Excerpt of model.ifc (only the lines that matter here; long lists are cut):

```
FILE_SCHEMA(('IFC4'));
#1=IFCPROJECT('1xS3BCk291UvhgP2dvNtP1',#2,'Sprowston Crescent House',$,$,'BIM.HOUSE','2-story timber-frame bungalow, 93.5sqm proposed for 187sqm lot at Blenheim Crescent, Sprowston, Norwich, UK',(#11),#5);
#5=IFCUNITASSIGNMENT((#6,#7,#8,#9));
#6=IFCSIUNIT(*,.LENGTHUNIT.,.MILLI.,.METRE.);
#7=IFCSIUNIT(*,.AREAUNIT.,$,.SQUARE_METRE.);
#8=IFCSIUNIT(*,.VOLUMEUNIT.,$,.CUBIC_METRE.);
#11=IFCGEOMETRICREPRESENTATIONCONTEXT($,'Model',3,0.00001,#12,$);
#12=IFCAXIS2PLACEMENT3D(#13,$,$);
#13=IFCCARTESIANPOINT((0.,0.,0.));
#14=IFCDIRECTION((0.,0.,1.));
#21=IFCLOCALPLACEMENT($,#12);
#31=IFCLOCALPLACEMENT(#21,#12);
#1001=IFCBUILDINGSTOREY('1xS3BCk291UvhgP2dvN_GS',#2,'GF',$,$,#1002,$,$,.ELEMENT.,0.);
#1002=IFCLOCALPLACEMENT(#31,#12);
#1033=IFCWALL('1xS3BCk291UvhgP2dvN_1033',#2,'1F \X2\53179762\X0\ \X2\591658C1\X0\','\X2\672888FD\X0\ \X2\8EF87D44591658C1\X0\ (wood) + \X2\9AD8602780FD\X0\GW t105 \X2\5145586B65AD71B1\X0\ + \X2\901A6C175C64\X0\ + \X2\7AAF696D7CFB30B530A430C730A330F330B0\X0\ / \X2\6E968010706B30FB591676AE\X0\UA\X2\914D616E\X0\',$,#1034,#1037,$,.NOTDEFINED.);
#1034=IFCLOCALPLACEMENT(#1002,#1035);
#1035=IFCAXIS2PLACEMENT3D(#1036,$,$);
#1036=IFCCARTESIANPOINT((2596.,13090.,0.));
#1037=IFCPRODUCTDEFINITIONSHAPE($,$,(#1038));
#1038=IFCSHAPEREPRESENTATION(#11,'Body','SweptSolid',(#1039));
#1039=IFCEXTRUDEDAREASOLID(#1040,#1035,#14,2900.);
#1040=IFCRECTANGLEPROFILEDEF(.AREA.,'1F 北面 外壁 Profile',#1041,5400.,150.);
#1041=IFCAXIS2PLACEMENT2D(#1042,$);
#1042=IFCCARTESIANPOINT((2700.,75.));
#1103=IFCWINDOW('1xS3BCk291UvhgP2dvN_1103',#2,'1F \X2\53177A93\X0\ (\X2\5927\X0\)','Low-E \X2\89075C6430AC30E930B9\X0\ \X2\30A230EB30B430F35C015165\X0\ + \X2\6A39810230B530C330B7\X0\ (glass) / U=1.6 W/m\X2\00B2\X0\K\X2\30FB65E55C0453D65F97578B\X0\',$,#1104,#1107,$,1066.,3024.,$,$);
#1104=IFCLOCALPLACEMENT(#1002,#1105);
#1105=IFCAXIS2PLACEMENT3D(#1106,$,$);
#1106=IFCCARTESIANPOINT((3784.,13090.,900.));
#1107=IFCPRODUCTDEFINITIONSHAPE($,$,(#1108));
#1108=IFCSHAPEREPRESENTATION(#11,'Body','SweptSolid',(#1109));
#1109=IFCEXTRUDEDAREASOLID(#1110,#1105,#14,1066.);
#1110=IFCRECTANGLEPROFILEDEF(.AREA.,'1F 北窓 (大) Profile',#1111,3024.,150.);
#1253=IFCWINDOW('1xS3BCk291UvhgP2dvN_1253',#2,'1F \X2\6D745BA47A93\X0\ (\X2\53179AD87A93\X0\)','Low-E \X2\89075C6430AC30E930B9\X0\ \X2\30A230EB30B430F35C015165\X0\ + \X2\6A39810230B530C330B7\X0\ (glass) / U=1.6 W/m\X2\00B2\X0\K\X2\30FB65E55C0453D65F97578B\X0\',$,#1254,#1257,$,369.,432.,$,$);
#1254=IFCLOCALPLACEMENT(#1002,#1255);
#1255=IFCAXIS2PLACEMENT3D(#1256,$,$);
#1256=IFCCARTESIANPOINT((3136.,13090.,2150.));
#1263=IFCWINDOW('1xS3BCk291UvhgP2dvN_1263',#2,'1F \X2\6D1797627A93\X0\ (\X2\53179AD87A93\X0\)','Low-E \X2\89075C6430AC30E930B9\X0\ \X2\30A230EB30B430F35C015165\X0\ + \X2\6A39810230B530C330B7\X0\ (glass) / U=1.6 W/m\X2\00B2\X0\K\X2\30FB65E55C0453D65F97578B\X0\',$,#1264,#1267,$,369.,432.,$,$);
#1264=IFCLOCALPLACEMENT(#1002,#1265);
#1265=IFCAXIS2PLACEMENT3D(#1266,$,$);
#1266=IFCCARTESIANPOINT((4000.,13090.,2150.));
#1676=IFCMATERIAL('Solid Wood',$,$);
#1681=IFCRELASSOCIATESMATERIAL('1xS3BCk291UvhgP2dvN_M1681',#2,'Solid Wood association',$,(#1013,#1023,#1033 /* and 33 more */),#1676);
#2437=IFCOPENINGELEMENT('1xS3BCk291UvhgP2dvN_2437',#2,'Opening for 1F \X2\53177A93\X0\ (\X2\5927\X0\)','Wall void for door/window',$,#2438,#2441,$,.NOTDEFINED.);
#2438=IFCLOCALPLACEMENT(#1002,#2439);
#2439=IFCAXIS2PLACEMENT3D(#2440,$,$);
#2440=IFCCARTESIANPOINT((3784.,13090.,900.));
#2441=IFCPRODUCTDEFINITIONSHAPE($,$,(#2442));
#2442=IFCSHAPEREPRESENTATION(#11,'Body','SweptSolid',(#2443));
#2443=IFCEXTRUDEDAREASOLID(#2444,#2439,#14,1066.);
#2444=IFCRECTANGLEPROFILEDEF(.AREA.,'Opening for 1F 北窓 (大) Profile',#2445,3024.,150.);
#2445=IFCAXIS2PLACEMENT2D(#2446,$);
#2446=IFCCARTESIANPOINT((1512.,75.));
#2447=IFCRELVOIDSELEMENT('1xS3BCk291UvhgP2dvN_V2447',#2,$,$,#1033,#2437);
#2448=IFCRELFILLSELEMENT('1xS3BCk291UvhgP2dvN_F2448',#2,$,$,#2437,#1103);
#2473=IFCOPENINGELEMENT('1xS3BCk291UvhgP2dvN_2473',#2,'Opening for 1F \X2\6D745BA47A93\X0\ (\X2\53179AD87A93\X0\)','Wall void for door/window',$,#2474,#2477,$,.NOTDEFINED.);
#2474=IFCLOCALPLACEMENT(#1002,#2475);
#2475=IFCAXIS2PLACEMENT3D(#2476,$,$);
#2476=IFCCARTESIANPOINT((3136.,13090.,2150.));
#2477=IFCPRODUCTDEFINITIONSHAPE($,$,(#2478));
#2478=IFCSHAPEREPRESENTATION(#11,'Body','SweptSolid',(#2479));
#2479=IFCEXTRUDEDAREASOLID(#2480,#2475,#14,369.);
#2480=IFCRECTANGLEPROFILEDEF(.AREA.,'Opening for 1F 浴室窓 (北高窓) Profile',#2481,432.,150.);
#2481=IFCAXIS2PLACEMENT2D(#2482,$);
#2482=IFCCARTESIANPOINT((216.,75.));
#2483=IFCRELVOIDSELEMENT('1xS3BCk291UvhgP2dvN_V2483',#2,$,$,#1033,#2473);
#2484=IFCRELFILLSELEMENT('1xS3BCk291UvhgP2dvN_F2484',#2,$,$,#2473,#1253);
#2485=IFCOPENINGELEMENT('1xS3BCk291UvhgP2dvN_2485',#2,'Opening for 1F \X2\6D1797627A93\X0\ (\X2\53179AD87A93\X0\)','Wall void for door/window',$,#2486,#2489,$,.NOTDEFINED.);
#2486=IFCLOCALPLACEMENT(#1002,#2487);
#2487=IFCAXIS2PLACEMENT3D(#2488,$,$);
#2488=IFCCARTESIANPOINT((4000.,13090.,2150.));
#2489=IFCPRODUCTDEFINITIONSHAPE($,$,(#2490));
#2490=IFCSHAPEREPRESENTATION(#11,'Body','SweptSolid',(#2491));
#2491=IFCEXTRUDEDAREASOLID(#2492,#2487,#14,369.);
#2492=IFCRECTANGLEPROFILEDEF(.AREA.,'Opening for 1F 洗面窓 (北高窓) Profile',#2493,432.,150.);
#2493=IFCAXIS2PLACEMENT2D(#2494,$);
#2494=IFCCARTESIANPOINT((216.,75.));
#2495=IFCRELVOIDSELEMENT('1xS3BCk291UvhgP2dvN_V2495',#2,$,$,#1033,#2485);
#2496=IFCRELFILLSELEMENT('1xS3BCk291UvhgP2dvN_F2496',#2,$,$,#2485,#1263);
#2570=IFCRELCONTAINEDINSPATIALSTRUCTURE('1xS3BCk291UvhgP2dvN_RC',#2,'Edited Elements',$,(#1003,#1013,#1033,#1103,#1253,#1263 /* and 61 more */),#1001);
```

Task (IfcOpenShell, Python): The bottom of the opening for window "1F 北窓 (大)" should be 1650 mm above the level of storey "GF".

```python
import numpy as np
import ifcopenshell
import ifcopenshell.api.geometry
import ifcopenshell.geom
import ifcopenshell.util.element
import ifcopenshell.util.placement
import ifcopenshell.util.shape
import ifcopenshell.util.unit

model = ifcopenshell.open("model.ifc")
unit_scale = ifcopenshell.util.unit.calculate_unit_scale(model)

window = model.by_guid("1xS3BCk291UvhgP2dvN_1103")
opening = window.FillsVoids[0].RelatingOpeningElement
storey = ifcopenshell.util.element.get_container(window, ifc_class="IfcBuildingStorey")
level = ifcopenshell.util.placement.get_local_placement(storey.ObjectPlacement)[2, 3]

# The opening's origin need not be at the sill, so measure its lowest point.
shape = ifcopenshell.geom.create_shape(ifcopenshell.geom.settings(), opening)
bottom = ifcopenshell.util.shape.get_shape_bottom_elevation(shape, shape.geometry) / unit_scale
dz = level + 1.65 / unit_scale - bottom

shift = np.array([0.0, 0.0, dz])
# The window is not placed relative to its opening, so move both.
for product in (opening, window):
    matrix = ifcopenshell.util.placement.get_local_placement(product.ObjectPlacement)
    matrix[:3, 3] += shift
    ifcopenshell.api.geometry.edit_object_placement(model, product=product, matrix=matrix, is_si=False)

print(f"moved by {dz * unit_scale:+.3f} m")

model.write("model_edited.ifc")
```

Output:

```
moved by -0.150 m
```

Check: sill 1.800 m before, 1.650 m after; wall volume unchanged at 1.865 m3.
